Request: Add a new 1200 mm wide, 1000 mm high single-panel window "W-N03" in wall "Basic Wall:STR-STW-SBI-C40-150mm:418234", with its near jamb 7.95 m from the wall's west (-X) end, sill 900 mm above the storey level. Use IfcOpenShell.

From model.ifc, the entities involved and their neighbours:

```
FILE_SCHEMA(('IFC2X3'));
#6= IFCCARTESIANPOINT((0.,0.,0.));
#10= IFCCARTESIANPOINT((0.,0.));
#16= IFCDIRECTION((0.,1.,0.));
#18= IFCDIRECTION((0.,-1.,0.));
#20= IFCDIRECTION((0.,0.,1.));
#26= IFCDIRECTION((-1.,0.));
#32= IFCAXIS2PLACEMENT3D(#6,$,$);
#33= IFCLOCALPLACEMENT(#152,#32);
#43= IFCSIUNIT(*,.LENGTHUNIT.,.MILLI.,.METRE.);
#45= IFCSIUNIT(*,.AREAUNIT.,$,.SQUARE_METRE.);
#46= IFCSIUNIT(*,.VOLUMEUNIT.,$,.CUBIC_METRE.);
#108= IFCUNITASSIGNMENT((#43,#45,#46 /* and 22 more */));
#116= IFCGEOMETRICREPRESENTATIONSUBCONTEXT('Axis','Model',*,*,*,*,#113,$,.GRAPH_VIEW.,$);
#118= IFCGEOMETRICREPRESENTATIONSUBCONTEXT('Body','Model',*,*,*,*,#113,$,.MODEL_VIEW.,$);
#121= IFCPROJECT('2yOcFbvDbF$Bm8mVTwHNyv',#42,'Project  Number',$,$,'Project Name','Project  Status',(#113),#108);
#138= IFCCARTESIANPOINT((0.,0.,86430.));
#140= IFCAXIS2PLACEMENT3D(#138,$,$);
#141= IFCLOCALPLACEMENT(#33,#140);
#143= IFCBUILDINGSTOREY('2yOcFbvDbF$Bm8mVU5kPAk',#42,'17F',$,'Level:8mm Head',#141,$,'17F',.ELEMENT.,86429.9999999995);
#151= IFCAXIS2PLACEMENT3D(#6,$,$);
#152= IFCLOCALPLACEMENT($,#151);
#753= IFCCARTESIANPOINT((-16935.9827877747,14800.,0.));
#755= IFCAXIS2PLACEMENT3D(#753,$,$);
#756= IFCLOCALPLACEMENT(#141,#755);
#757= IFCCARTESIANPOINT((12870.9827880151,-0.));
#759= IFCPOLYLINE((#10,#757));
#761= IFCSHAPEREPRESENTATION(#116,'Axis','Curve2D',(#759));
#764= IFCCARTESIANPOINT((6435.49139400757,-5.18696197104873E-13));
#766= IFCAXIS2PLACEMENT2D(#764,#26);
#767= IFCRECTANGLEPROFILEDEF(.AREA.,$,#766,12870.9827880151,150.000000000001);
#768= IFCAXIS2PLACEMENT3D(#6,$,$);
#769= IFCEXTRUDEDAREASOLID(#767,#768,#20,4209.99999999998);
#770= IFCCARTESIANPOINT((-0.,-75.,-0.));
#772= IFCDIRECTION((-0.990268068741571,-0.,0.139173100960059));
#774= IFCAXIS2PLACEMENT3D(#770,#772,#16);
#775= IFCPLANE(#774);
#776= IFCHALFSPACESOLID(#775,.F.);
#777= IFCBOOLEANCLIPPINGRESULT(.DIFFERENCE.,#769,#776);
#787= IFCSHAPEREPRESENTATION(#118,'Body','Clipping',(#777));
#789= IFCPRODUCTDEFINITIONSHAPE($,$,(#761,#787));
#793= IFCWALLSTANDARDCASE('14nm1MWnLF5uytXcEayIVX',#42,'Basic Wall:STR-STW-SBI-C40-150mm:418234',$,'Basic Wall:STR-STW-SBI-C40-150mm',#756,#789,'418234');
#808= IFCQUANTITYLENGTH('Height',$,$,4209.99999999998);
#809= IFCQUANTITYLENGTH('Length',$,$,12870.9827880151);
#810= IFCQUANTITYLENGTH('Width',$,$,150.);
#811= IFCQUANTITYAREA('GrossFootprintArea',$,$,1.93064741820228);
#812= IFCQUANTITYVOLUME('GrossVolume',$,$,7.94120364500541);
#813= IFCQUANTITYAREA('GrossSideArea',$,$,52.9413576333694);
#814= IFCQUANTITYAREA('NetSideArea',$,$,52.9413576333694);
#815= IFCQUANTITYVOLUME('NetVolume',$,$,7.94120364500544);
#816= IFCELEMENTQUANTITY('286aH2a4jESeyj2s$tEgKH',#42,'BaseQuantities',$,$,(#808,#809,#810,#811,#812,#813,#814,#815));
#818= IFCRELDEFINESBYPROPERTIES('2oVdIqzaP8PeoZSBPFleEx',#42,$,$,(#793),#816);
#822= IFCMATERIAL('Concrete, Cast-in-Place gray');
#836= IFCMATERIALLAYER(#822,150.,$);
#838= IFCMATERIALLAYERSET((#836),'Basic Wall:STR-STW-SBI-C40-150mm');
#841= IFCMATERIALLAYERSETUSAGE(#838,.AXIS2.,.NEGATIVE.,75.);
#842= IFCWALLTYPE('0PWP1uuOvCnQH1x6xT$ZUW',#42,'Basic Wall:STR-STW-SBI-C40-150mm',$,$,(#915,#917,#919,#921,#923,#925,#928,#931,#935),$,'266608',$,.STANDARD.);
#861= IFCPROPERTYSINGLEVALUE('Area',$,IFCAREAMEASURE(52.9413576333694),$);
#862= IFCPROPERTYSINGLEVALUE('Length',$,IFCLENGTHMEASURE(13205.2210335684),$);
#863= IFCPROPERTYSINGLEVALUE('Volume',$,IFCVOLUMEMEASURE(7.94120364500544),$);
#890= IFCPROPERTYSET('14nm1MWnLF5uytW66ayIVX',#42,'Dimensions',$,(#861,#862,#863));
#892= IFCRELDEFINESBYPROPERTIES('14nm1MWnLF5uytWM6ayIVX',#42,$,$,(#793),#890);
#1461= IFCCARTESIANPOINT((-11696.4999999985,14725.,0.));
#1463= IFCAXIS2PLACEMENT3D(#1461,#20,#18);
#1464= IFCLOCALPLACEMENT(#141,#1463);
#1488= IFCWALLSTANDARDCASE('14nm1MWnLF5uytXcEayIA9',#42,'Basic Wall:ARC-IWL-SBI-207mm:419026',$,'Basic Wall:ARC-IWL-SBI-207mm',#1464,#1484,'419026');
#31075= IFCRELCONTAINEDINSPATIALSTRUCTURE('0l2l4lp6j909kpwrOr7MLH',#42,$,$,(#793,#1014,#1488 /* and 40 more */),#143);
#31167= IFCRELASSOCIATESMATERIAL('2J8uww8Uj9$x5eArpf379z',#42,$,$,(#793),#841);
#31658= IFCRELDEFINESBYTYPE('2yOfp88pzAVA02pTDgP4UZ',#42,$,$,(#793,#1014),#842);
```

```python
import numpy as np
import ifcopenshell
import ifcopenshell.api.feature
import ifcopenshell.api.geometry
import ifcopenshell.api.pset
import ifcopenshell.api.root
import ifcopenshell.api.spatial
import ifcopenshell.api.type
import ifcopenshell.geom
import ifcopenshell.util.element
import ifcopenshell.util.placement
import ifcopenshell.util.representation
import ifcopenshell.util.shape
import ifcopenshell.util.unit

model = ifcopenshell.open("model.ifc")
unit_scale = ifcopenshell.util.unit.calculate_unit_scale(model)
area_scale = ifcopenshell.util.unit.calculate_unit_scale(model, "AREAUNIT")
volume_scale = ifcopenshell.util.unit.calculate_unit_scale(model, "VOLUMEUNIT")
settings = ifcopenshell.geom.settings()


def volume(element):
    """Net volume in cubic metres, openings subtracted."""
    shape = ifcopenshell.geom.create_shape(settings, element)
    return ifcopenshell.util.shape.get_volume(shape.geometry)


wall = model.by_guid("14nm1MWnLF5uytXcEayIVX")
storey = ifcopenshell.util.element.get_container(wall, ifc_class="IfcBuildingStorey")
context = ifcopenshell.util.representation.get_context(model, "Model", "Body", "MODEL_VIEW")
before = volume(wall)

width, height, from_end, sill = 1.2, 1, 7.95, 0.9  # metres

# The wall runs along its own X axis, and the end named is its -X end.
wall_shape = ifcopenshell.geom.create_shape(settings, wall)
x, y, z = ifcopenshell.util.shape.get_vertices(wall_shape.geometry).T
start = x.min() + from_end
face, thickness = float(y.min()), float(y.max() - y.min())
wall_matrix = ifcopenshell.util.placement.get_local_placement(wall.ObjectPlacement)
level = ifcopenshell.util.placement.get_local_placement(storey.ObjectPlacement)[2, 3]


def in_wall(x, y):
    """Placement at x, y metres in the wall's axes, at sill height."""
    matrix = wall_matrix.copy()
    matrix[:, 3] = wall_matrix @ np.array([x / unit_scale, y / unit_scale, 0.0, 1.0])
    matrix[2, 3] = level + sill / unit_scale
    return matrix


# Opening: a box that overshoots both wall faces by 50 mm.
opening = ifcopenshell.api.root.create_entity(model, ifc_class="IfcOpeningElement")
box = ifcopenshell.api.geometry.add_wall_representation(
    model, context=context, length=width, height=height, thickness=thickness + 0.1
)
ifcopenshell.api.geometry.assign_representation(model, product=opening, representation=box)
ifcopenshell.api.geometry.edit_object_placement(model, product=opening, matrix=in_wall(start, face - 0.05), is_si=False)
ifcopenshell.api.feature.add_feature(model, feature=opening, element=wall)

window = ifcopenshell.api.root.create_entity(model, ifc_class="IfcWindow", name="W-N03")
window.OverallWidth, window.OverallHeight = width / unit_scale, height / unit_scale
body = ifcopenshell.api.geometry.add_window_representation(
    model,
    context=context,
    overall_width=window.OverallWidth,
    overall_height=window.OverallHeight,
    partition_type="SINGLE_PANEL",
)
ifcopenshell.api.geometry.assign_representation(model, product=window, representation=body)
ifcopenshell.api.spatial.assign_container(model, products=[window], relating_structure=storey)
fills = ifcopenshell.api.feature.add_filling(model, opening=opening, element=window)
fills.OwnerHistory = window.OwnerHistory  # required in IFC2X3

# IFC2X3 keeps the operation on the window style.
style = ifcopenshell.api.root.create_entity(model, ifc_class="IfcWindowStyle", name="W-N03")
style.OperationType, style.ConstructionType = "SINGLE_PANEL", "NOTDEFINED"
style.ParameterTakesPrecedence = style.Sizeable = False
ifcopenshell.api.type.assign_type(model, related_objects=[window], relating_type=style)

# Centre the window in the wall's thickness.
ifcopenshell.api.geometry.edit_object_placement(model, product=window, matrix=in_wall(start, face), is_si=False)
window_shape = ifcopenshell.geom.create_shape(settings, window)
depth = ifcopenshell.util.shape.get_vertices(window_shape.geometry)[:, 1]
offset = face + thickness / 2 - (depth.min() + depth.max()) / 2
ifcopenshell.api.geometry.edit_object_placement(model, product=window, matrix=in_wall(start, offset), is_si=False)

after = volume(wall)

# Update the wall's stored quantities.
qto = model.by_id(ifcopenshell.util.element.get_pset(wall, "BaseQuantities", should_inherit=False)["id"])
ifcopenshell.api.pset.edit_qto(model, qto=qto, properties={
    "NetSideArea": after / thickness / area_scale,
    "NetVolume": after / volume_scale,
})
pset = model.by_id(ifcopenshell.util.element.get_pset(wall, "Dimensions", should_inherit=False)["id"])
ifcopenshell.api.pset.edit_pset(model, pset=pset, properties={
    "Area": model.create_entity("IfcAreaMeasure", after / thickness / area_scale),
    "Volume": model.create_entity("IfcVolumeMeasure", after / volume_scale),
})

print(f"wall volume {before:.3f} -> {after:.3f} m3")

model.write("model_rev.ifc")
```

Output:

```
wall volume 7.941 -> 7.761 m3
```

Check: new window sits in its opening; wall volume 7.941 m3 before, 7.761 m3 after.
